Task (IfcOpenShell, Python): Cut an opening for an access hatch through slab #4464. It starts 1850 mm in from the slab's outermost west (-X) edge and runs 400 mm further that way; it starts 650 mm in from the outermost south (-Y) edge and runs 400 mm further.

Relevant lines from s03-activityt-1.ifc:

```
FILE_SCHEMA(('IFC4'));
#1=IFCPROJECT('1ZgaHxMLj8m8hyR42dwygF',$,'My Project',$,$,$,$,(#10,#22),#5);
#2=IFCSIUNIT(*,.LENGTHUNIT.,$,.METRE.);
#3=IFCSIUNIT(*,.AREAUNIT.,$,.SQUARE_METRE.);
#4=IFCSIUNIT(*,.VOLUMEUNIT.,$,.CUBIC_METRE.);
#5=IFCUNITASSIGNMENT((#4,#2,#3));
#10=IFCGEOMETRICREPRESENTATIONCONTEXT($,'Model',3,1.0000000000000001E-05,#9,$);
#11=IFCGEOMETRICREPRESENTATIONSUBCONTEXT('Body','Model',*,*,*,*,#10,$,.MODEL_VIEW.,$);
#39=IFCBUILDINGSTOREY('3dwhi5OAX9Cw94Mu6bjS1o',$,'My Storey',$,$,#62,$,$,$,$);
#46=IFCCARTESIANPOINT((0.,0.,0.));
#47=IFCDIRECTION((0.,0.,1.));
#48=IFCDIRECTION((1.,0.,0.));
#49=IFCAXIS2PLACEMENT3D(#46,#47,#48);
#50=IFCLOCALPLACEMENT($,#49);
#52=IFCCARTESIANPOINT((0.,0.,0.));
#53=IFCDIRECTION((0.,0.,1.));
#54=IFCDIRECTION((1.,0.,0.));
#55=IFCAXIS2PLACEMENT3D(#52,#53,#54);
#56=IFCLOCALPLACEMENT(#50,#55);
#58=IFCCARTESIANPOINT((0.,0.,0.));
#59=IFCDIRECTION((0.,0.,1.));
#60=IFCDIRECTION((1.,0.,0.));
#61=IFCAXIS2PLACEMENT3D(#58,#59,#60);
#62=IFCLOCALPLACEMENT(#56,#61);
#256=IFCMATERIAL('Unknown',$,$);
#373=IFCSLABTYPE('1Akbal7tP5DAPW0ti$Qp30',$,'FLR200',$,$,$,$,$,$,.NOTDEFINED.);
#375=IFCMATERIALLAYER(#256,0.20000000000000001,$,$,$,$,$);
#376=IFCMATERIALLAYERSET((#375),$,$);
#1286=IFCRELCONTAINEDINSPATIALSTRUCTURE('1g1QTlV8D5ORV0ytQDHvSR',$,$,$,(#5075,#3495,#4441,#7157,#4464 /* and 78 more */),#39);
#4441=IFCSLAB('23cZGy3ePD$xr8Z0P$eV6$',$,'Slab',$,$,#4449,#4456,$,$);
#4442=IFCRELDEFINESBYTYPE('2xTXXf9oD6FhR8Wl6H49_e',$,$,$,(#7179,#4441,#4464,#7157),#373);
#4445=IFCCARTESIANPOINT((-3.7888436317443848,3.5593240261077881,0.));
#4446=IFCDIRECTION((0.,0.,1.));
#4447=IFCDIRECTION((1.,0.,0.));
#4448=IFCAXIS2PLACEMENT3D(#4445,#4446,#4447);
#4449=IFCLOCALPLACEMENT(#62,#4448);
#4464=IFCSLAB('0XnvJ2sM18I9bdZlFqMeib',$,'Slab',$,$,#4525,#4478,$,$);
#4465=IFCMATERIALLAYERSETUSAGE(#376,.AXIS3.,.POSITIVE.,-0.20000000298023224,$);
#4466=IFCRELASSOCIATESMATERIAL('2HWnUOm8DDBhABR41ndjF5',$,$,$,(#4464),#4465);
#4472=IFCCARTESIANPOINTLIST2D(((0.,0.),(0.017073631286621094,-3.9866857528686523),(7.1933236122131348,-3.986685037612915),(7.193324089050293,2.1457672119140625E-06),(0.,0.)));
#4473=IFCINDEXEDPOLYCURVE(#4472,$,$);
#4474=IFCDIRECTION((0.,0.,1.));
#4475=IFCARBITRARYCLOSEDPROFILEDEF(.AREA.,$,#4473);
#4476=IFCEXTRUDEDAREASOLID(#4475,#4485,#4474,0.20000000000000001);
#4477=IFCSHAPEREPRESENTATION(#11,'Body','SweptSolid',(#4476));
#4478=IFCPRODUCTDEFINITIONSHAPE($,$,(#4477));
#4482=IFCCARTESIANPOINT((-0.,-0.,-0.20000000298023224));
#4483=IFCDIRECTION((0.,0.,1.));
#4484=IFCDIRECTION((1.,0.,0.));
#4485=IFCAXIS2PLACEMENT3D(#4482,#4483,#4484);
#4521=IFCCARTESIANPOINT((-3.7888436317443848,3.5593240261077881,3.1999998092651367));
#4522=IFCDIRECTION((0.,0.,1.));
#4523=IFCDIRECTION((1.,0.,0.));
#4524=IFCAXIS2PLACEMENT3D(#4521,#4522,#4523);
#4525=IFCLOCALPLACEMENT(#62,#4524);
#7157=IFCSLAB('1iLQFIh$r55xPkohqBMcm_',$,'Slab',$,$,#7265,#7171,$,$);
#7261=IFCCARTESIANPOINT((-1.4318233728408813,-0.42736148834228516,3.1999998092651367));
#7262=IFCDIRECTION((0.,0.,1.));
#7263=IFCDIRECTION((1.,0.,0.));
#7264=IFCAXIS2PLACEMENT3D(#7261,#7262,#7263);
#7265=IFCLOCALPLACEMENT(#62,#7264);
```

```python
import numpy as np
import ifcopenshell
import ifcopenshell.api.feature
import ifcopenshell.api.geometry
import ifcopenshell.api.root
import ifcopenshell.geom
import ifcopenshell.util.placement
import ifcopenshell.util.representation
import ifcopenshell.util.shape
import ifcopenshell.util.unit

model = ifcopenshell.open("s03-activityt-1.ifc")
unit_scale = ifcopenshell.util.unit.calculate_unit_scale(model)
settings = ifcopenshell.geom.settings()


def volume(element):
    """Net volume in cubic metres, openings subtracted."""
    shape = ifcopenshell.geom.create_shape(settings, element)
    return ifcopenshell.util.shape.get_volume(shape.geometry)


slab = model.by_guid("0XnvJ2sM18I9bdZlFqMeib")
before = volume(slab)

# Extent in the slab's own axes, in metres. The edges named are its -X and -Y sides.
slab_shape = ifcopenshell.geom.create_shape(settings, slab)
vertices = ifcopenshell.util.shape.get_vertices(slab_shape.geometry)
x_min, y_min, bottom = vertices.min(axis=0)
top = vertices[:, 2].max()

opening = ifcopenshell.api.root.create_entity(model, ifc_class="IfcOpeningElement", name="Access hatch opening", predefined_type="OPENING")
context = ifcopenshell.util.representation.get_context(model, "Model", "Body", "MODEL_VIEW")
width, depth = 0.4, 0.4
outline = [(0.0, 0.0), (width, 0.0), (width, depth), (0.0, depth), (0.0, 0.0)]
# Overshoot both faces by 50 mm so the cut is clean.
shape = ifcopenshell.api.geometry.add_slab_representation(
    model, context=context, depth=top - bottom + 0.1, polyline=outline
)
ifcopenshell.api.geometry.assign_representation(model, product=opening, representation=shape)

matrix = ifcopenshell.util.placement.get_local_placement(slab.ObjectPlacement)
matrix[:, 3] = matrix @ np.append(np.array([x_min + 1.85, y_min + 0.65, bottom - 0.05]) / unit_scale, 1.0)
ifcopenshell.api.geometry.edit_object_placement(model, product=opening, matrix=matrix, is_si=False)
ifcopenshell.api.feature.add_feature(model, feature=opening, element=slab)

after = volume(slab)

print(f"slab volume {before:.3f} -> {after:.3f} m3")

model.write("s03-activityt-1_rev.ifc")
```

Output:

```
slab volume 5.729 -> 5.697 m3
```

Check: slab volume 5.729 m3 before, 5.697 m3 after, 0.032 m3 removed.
